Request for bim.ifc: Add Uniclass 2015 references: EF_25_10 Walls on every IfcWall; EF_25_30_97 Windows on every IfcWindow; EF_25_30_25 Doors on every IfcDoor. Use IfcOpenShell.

First a look at what the model holds.

```python
import ifcopenshell

model = ifcopenshell.open("bim.ifc")
print(model.schema)
print("classifications:", [c.Name for c in model.by_type("IfcClassification")])
for ifc_class in ("IfcDoor", "IfcRoof", "IfcStair", "IfcWall", "IfcWindow"):
    print(ifc_class, len(model.by_type(ifc_class)))
```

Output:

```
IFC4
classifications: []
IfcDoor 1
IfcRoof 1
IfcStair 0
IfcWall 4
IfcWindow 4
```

```python
import ifcopenshell
import ifcopenshell.api.classification

model = ifcopenshell.open("bim.ifc")

system = ifcopenshell.api.classification.add_classification(model, classification="Uniclass 2015")

codes = {
    "IfcWall": ("EF_25_10", "Walls"),
    "IfcWindow": ("EF_25_30_97", "Windows"),
    "IfcDoor": ("EF_25_30_25", "Doors"),
}
for ifc_class, (code, name) in codes.items():
    products = model.by_type(ifc_class)
    ifcopenshell.api.classification.add_reference(
        model, products=products, classification=system, identification=code, name=name
    )
    print(code, len(products))

model.write("bim_updated.ifc")
```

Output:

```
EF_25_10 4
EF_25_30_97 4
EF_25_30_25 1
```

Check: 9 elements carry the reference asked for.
